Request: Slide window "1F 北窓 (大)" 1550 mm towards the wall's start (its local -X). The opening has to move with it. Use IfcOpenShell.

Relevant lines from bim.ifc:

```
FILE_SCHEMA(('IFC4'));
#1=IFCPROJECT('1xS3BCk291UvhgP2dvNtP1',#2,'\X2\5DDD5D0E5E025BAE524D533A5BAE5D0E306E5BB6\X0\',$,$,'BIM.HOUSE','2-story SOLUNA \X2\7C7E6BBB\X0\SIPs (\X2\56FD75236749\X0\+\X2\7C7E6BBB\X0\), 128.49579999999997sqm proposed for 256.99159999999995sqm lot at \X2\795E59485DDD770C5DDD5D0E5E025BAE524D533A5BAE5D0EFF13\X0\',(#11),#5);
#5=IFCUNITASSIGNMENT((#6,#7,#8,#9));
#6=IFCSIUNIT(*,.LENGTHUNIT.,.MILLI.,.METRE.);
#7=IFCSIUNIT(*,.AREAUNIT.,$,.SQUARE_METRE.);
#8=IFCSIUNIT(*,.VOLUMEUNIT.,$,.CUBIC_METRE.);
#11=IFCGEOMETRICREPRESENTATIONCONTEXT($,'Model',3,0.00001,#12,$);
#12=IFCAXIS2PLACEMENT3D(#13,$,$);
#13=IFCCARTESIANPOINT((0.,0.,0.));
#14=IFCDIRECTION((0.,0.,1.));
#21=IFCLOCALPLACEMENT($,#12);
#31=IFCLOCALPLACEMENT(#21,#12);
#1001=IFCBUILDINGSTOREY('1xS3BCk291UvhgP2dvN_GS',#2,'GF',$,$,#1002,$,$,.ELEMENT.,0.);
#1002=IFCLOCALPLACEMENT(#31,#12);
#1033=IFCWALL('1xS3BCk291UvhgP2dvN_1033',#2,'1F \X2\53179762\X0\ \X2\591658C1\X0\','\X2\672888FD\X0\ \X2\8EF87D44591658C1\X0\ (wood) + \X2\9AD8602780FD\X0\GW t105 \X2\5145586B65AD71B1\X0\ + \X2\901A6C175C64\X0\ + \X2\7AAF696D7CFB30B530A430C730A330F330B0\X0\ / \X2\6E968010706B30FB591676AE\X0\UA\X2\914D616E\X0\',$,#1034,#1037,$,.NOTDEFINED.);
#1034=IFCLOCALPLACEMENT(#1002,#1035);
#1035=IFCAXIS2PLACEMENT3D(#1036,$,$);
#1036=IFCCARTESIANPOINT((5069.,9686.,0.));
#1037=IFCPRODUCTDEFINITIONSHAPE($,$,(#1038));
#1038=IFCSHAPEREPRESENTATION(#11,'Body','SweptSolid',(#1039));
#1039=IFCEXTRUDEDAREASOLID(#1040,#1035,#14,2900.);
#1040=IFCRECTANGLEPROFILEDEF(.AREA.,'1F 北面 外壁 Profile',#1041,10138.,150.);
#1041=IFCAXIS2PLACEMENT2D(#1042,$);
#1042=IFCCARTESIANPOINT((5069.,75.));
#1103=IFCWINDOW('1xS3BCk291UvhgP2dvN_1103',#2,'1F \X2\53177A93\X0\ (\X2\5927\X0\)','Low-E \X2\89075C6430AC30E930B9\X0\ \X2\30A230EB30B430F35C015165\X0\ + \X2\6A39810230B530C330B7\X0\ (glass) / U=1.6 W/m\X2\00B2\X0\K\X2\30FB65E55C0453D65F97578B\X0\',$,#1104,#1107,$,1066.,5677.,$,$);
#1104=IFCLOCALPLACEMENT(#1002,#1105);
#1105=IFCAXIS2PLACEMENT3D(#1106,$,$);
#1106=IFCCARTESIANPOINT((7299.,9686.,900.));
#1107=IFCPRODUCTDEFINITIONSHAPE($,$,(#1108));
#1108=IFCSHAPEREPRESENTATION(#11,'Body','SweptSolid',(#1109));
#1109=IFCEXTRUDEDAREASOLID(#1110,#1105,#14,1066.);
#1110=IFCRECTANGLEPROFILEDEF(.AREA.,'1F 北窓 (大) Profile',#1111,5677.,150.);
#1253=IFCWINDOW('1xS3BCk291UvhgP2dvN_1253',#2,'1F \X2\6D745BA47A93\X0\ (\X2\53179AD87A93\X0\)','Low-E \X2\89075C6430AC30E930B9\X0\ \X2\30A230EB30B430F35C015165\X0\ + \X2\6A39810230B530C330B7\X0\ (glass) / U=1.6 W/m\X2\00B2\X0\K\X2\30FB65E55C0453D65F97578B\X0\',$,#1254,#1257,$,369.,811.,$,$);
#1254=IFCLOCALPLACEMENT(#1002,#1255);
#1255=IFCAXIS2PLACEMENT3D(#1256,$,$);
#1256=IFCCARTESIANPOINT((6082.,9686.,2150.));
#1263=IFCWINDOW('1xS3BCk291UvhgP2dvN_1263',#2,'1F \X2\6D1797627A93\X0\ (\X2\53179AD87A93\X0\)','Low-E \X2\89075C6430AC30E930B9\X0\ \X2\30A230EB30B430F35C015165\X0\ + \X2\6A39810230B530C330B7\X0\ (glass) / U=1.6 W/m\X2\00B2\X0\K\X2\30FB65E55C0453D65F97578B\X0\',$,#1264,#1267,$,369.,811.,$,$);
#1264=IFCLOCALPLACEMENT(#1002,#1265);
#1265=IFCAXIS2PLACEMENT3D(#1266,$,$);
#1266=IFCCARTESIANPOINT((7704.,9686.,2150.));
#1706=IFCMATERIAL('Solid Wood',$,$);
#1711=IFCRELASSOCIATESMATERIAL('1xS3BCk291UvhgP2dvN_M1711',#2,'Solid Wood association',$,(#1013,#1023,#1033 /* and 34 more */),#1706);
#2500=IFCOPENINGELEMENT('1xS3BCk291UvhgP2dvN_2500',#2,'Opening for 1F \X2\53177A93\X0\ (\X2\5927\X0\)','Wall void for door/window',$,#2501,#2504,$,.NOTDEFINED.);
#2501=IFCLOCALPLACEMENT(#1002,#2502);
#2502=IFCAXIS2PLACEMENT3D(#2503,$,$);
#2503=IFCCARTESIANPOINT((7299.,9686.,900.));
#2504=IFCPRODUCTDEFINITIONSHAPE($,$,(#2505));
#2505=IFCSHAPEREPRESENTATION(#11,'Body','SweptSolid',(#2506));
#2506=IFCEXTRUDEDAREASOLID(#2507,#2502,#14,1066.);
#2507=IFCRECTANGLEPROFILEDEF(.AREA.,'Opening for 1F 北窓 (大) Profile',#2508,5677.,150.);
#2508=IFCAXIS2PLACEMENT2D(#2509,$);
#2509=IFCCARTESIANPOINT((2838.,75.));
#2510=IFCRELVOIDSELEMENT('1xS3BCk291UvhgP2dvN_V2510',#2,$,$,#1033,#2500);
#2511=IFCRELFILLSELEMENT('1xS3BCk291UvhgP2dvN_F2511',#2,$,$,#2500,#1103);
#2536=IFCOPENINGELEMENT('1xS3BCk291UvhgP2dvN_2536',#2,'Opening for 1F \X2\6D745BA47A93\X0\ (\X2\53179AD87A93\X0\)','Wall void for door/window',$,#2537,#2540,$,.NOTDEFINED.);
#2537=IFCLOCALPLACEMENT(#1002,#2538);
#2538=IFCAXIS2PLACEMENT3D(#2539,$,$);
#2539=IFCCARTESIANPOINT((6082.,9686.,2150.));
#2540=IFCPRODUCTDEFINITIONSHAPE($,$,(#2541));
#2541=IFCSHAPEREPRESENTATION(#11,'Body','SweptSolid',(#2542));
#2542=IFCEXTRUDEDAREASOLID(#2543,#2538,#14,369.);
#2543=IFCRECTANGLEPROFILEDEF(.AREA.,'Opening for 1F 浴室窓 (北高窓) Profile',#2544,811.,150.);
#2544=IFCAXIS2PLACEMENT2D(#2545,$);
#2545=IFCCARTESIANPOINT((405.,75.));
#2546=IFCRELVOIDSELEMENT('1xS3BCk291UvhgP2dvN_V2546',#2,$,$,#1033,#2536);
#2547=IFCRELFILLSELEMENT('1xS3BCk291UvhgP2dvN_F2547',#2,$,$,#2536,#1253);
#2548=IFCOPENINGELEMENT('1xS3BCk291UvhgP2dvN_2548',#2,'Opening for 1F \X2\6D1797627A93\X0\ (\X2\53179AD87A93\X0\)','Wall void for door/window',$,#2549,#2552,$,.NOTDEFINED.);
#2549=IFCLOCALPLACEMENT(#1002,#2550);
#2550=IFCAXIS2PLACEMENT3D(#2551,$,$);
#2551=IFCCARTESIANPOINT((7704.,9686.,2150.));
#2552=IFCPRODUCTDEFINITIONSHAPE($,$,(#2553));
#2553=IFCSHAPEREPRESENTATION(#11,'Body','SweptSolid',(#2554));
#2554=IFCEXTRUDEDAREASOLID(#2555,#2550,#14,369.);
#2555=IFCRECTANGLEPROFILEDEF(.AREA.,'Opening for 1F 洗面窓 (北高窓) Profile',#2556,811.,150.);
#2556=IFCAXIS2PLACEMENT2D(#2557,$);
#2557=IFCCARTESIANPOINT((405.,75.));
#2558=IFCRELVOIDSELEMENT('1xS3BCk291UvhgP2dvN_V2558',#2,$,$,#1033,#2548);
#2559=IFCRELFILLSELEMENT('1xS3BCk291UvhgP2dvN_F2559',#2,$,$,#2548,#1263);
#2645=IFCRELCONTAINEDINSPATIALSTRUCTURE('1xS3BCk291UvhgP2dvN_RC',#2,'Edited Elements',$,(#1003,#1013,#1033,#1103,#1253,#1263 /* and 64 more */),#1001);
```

```python
import ifcopenshell
import ifcopenshell.api.geometry
import ifcopenshell.util.placement

model = ifcopenshell.open("bim.ifc")

window = model.by_guid("1xS3BCk291UvhgP2dvN_1103")
opening = window.FillsVoids[0].RelatingOpeningElement
wall = opening.VoidsElements[0].RelatingBuildingElement

wall_matrix = ifcopenshell.util.placement.get_local_placement(wall.ObjectPlacement)
shift = wall_matrix[:3, 0] * -1550.0
before = ifcopenshell.util.placement.get_local_placement(window.ObjectPlacement)[:3, 3].copy()

# The window is not placed relative to its opening, so move both.
for product in (opening, window):
    matrix = ifcopenshell.util.placement.get_local_placement(product.ObjectPlacement)
    matrix[:3, 3] += shift
    ifcopenshell.api.geometry.edit_object_placement(model, product=product, matrix=matrix, is_si=False)

after = ifcopenshell.util.placement.get_local_placement(window.ObjectPlacement)[:3, 3]
print("window moved by", (after - before).round(3) + 0.0)

model.write("bim_v2.ifc")
```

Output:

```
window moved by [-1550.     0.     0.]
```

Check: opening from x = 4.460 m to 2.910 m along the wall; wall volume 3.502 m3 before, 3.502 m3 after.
